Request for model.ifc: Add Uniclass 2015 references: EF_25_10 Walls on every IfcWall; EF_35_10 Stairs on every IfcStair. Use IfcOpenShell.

First a look at what the model holds.

```python
import ifcopenshell

model = ifcopenshell.open("model.ifc")
print(model.schema)
print("classifications:", [c.Name for c in model.by_type("IfcClassification")])
for ifc_class in ("IfcDoor", "IfcRoof", "IfcStair", "IfcWall", "IfcWindow"):
    print(ifc_class, len(model.by_type(ifc_class)))
```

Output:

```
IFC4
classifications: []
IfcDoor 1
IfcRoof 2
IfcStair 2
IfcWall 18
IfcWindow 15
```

```python
import ifcopenshell
import ifcopenshell.api.classification

model = ifcopenshell.open("model.ifc")

system = ifcopenshell.api.classification.add_classification(model, classification="Uniclass 2015")

codes = {
    "IfcWall": ("EF_25_10", "Walls"),
    "IfcStair": ("EF_35_10", "Stairs"),
}
for ifc_class, (code, name) in codes.items():
    products = model.by_type(ifc_class)
    ifcopenshell.api.classification.add_reference(
        model, products=products, classification=system, identification=code, name=name
    )
    print(code, len(products))

model.write("model-out.ifc")
```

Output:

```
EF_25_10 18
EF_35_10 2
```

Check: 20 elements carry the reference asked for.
